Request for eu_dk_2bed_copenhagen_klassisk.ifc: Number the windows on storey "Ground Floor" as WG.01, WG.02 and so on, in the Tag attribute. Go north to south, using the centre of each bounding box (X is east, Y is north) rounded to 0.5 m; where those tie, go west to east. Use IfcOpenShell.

First a look at what the model holds.

```python
import ifcopenshell
import ifcopenshell.util.element
import ifcopenshell.util.placement

model = ifcopenshell.open("eu_dk_2bed_copenhagen_klassisk.ifc")
print(model.schema)
storey = next(s for s in model.by_type("IfcBuildingStorey") if s.Name == "Ground Floor")
windows = [e for e in ifcopenshell.util.element.get_decomposition(storey) if e.is_a("IfcWindow")]
for e in sorted(windows, key=lambda e: e.id()):
    origin = ifcopenshell.util.placement.get_local_placement(e.ObjectPlacement)[:3, 3]
    print(e.id(), e.Tag, e.Name, origin.round(2) + 0.0, sep=" | ")
```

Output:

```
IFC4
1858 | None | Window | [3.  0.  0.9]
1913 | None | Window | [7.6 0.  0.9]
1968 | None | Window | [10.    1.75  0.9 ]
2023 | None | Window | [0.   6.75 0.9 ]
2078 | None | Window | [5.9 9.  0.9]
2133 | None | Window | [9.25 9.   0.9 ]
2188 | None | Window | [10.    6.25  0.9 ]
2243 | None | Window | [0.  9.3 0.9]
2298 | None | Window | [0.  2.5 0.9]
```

```python
import ifcopenshell
import ifcopenshell.geom
import ifcopenshell.util.element
import ifcopenshell.util.shape

model = ifcopenshell.open("eu_dk_2bed_copenhagen_klassisk.ifc")
settings = ifcopenshell.geom.settings()
settings.set("use-world-coords", True)


def centre(element):
    shape = ifcopenshell.geom.create_shape(settings, element)
    return ifcopenshell.util.shape.get_bbox_centroid(shape.geometry)


storey = next(s for s in model.by_type("IfcBuildingStorey") if s.Name == "Ground Floor")
windows = [e for e in ifcopenshell.util.element.get_decomposition(storey) if e.is_a("IfcWindow")]

# Insertion points can sit at a corner or the storey origin, so sort by the geometry (in metres).
centres = {e: centre(e) for e in windows}
windows.sort(key=lambda e: (-round(centres[e][1] / 0.5), centres[e][0]))

for i, e in enumerate(windows, start=1):
    number = f"WG.{i:02d}"
    e.Tag = number
    print(e.id(), number)

model.write("eu_dk_2bed_copenhagen_klassisk-out.ifc")
```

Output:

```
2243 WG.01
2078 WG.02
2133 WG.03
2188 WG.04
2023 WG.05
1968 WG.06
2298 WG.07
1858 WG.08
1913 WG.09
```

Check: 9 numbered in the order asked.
